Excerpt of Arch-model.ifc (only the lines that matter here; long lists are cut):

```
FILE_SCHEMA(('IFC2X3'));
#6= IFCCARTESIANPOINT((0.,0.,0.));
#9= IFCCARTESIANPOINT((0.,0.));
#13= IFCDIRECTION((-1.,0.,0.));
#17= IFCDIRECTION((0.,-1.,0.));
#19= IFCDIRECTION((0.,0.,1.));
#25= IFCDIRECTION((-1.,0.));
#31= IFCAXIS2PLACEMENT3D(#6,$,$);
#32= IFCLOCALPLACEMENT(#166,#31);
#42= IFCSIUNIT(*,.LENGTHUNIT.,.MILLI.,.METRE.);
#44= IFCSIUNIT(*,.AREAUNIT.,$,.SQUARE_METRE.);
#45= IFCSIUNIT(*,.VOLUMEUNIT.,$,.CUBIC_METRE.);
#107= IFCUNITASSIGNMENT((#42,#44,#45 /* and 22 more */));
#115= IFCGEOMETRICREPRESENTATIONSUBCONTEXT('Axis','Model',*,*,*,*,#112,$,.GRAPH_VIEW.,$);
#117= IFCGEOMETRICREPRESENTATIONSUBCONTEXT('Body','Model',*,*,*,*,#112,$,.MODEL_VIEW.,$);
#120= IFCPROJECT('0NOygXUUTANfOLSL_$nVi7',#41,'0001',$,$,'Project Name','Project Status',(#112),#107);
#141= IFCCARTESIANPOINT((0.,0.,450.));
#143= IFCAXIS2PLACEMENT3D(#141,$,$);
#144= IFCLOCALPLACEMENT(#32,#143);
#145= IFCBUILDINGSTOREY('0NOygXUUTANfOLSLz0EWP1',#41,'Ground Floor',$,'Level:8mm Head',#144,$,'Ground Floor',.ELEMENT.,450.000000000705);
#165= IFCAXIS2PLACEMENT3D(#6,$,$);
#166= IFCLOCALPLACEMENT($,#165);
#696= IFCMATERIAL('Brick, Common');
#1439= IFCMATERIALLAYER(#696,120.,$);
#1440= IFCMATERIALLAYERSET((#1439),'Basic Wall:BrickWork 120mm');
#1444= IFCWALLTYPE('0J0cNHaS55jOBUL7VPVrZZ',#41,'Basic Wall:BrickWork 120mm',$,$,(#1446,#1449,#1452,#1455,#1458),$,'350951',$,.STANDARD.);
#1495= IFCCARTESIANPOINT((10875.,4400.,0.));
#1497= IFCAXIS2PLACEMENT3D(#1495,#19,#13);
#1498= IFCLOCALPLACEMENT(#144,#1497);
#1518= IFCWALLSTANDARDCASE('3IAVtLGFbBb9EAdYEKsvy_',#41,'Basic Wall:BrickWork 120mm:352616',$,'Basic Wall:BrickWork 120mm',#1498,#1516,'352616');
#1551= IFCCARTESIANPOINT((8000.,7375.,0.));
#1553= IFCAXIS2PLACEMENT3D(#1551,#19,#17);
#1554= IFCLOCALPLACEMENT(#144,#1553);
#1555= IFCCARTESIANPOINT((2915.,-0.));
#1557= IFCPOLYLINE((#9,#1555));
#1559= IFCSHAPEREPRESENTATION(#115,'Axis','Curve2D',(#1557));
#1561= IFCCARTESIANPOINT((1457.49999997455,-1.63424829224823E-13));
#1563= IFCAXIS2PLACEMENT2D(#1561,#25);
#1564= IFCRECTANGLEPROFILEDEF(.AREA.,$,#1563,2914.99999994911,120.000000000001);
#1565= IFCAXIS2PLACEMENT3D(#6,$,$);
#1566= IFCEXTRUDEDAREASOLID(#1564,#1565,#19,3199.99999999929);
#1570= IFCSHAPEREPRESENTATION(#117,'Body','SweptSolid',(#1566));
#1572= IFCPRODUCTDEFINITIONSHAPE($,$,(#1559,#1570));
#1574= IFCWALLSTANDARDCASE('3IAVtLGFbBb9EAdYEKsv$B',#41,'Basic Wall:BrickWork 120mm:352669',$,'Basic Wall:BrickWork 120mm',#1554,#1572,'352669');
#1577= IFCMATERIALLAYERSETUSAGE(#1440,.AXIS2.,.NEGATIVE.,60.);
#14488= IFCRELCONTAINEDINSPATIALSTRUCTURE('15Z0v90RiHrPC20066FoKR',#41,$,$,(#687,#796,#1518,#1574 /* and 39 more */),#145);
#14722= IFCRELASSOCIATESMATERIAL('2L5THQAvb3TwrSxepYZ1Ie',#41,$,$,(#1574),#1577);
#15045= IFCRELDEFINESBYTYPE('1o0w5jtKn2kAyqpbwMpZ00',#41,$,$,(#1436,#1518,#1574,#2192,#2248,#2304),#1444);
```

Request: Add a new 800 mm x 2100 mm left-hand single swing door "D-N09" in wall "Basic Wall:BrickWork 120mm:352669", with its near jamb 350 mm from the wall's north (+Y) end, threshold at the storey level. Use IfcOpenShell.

```python
import numpy as np
import ifcopenshell
import ifcopenshell.api.feature
import ifcopenshell.api.geometry
import ifcopenshell.api.root
import ifcopenshell.api.spatial
import ifcopenshell.api.type
import ifcopenshell.geom
import ifcopenshell.util.element
import ifcopenshell.util.placement
import ifcopenshell.util.representation
import ifcopenshell.util.shape
import ifcopenshell.util.unit

model = ifcopenshell.open("Arch-model.ifc")
unit_scale = ifcopenshell.util.unit.calculate_unit_scale(model)
settings = ifcopenshell.geom.settings()


def volume(element):
    """Net volume in cubic metres, openings subtracted."""
    shape = ifcopenshell.geom.create_shape(settings, element)
    return ifcopenshell.util.shape.get_volume(shape.geometry)


wall = model.by_id(1574)
storey = ifcopenshell.util.element.get_container(wall, ifc_class="IfcBuildingStorey")
context = ifcopenshell.util.representation.get_context(model, "Model", "Body", "MODEL_VIEW")
before = volume(wall)

width, height, from_end, sill = 0.8, 2.1, 0.35, 0.0  # metres

# The wall runs along its own X axis, and the end named is its -X end.
wall_shape = ifcopenshell.geom.create_shape(settings, wall)
x, y, z = ifcopenshell.util.shape.get_vertices(wall_shape.geometry).T
start = x.min() + from_end
face, thickness = float(y.min()), float(y.max() - y.min())
wall_matrix = ifcopenshell.util.placement.get_local_placement(wall.ObjectPlacement)
level = ifcopenshell.util.placement.get_local_placement(storey.ObjectPlacement)[2, 3]


def in_wall(x, y):
    """Placement at x, y metres in the wall's axes, at sill height."""
    matrix = wall_matrix.copy()
    matrix[:, 3] = wall_matrix @ np.array([x / unit_scale, y / unit_scale, 0.0, 1.0])
    matrix[2, 3] = level + sill / unit_scale
    return matrix


# Opening: a box that overshoots both wall faces by 50 mm.
opening = ifcopenshell.api.root.create_entity(model, ifc_class="IfcOpeningElement")
box = ifcopenshell.api.geometry.add_wall_representation(
    model, context=context, length=width, height=height, thickness=thickness + 0.1
)
ifcopenshell.api.geometry.assign_representation(model, product=opening, representation=box)
ifcopenshell.api.geometry.edit_object_placement(model, product=opening, matrix=in_wall(start, face - 0.05), is_si=False)
ifcopenshell.api.feature.add_feature(model, feature=opening, element=wall)

door = ifcopenshell.api.root.create_entity(model, ifc_class="IfcDoor", name="D-N09")
door.OverallWidth, door.OverallHeight = width / unit_scale, height / unit_scale
body = ifcopenshell.api.geometry.add_door_representation(
    model,
    context=context,
    overall_width=door.OverallWidth,
    overall_height=door.OverallHeight,
    operation_type="SINGLE_SWING_LEFT",
    lining_properties={"LiningDepth": thickness / unit_scale, "ThresholdDepth": thickness / unit_scale},
)
ifcopenshell.api.geometry.assign_representation(model, product=door, representation=body)
ifcopenshell.api.spatial.assign_container(model, products=[door], relating_structure=storey)
fills = ifcopenshell.api.feature.add_filling(model, opening=opening, element=door)
fills.OwnerHistory = door.OwnerHistory  # required in IFC2X3

# IFC2X3 keeps the operation on the door style.
style = ifcopenshell.api.root.create_entity(model, ifc_class="IfcDoorStyle", name="D-N09")
style.OperationType, style.ConstructionType = "SINGLE_SWING_LEFT", "NOTDEFINED"
style.ParameterTakesPrecedence = style.Sizeable = False
ifcopenshell.api.type.assign_type(model, related_objects=[door], relating_type=style)

# The lining spans the wall, so the door starts at the wall face.
ifcopenshell.api.geometry.edit_object_placement(model, product=door, matrix=in_wall(start, face), is_si=False)

after = volume(wall)

print(f"wall volume {before:.3f} -> {after:.3f} m3")

model.write("Arch-model_updated.ifc")
```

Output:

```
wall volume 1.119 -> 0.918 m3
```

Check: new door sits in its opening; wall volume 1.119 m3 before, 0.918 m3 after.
